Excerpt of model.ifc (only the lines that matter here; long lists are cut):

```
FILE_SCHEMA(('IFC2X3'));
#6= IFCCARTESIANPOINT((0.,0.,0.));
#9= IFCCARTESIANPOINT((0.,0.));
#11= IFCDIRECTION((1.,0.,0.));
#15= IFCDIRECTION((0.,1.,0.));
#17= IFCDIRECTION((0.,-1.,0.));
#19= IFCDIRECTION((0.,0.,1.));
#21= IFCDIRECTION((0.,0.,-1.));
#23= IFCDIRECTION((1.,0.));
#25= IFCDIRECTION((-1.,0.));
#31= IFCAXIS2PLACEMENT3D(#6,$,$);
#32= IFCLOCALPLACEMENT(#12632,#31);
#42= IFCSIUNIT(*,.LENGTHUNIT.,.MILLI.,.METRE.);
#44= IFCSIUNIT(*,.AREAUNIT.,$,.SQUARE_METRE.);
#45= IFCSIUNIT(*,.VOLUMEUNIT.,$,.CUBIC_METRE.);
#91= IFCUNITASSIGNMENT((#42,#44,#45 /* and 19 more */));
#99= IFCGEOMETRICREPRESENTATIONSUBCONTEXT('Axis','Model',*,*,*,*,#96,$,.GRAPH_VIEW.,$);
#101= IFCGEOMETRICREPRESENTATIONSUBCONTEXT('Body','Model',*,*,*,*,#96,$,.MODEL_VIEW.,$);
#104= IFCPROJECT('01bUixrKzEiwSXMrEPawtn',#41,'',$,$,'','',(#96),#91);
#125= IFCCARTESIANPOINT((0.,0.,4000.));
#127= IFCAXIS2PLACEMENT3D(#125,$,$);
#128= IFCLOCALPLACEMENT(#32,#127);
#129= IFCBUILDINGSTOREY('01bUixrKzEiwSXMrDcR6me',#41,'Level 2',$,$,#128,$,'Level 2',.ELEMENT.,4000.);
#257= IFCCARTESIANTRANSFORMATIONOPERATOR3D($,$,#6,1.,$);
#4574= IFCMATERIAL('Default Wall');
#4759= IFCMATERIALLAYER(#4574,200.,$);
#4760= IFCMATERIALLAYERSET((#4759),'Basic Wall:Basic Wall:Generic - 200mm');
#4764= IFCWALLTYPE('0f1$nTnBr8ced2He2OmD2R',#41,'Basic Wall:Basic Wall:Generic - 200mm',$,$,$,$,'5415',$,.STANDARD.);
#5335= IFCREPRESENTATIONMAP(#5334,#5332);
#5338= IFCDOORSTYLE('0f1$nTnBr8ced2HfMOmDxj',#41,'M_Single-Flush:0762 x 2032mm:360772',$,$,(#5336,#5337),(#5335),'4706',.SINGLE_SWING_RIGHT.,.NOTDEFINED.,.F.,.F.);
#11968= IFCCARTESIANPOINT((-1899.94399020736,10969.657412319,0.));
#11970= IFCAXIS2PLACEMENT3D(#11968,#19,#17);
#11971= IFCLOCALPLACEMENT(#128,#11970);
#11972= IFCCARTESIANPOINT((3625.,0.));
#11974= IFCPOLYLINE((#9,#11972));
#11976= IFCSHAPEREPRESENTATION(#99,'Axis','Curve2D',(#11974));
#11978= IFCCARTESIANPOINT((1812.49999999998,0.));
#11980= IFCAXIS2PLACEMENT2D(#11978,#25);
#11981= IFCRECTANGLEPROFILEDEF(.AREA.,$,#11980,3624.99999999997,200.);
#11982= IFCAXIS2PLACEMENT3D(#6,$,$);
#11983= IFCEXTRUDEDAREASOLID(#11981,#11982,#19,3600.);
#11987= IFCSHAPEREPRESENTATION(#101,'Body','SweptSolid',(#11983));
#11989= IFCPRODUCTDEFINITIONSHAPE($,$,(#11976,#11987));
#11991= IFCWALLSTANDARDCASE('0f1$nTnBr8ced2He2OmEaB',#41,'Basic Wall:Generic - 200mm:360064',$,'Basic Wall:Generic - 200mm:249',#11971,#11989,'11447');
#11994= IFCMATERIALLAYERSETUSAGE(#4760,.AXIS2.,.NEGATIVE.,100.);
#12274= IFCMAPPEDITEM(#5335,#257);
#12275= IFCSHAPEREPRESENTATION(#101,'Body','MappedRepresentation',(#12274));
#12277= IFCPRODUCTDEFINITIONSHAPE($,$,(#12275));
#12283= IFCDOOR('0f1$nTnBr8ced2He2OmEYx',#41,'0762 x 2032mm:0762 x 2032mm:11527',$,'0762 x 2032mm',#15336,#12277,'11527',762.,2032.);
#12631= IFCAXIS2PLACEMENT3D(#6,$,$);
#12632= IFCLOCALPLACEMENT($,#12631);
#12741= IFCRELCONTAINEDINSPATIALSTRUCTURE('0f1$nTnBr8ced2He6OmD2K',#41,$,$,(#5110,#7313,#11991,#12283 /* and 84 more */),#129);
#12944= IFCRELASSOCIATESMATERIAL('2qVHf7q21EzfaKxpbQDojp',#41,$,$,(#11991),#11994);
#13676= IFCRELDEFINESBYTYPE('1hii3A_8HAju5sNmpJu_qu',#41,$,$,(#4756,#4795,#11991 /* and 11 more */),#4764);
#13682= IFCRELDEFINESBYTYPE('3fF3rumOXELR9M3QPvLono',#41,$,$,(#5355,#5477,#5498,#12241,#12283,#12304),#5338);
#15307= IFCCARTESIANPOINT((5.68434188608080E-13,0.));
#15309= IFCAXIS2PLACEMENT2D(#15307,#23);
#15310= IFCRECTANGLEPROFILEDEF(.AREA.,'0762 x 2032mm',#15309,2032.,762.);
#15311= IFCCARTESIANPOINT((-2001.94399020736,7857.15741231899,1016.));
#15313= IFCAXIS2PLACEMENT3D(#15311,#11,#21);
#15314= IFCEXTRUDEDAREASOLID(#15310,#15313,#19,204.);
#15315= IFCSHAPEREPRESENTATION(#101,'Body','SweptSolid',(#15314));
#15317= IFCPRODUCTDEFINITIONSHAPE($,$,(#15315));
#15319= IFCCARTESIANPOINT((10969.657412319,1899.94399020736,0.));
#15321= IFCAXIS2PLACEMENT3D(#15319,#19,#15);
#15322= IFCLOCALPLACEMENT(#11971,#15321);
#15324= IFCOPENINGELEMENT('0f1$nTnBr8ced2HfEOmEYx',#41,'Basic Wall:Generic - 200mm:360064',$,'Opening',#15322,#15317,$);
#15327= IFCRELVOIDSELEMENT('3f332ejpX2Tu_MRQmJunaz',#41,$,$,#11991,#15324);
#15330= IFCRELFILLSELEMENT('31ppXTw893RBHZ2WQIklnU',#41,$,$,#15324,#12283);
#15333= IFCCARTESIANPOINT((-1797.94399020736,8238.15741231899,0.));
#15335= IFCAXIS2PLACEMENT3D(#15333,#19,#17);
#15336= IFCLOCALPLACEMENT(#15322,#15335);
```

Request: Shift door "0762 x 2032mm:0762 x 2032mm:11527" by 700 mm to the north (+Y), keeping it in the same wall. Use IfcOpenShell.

```python
import ifcopenshell
import ifcopenshell.api.geometry
import ifcopenshell.util.placement
import ifcopenshell.util.unit

model = ifcopenshell.open("model.ifc")
unit_scale = ifcopenshell.util.unit.calculate_unit_scale(model)

door = model.by_id(12283)
opening = door.FillsVoids[0].RelatingOpeningElement
wall = opening.VoidsElements[0].RelatingBuildingElement

wall_matrix = ifcopenshell.util.placement.get_local_placement(wall.ObjectPlacement)
shift = wall_matrix[:3, 0] * -0.7 / unit_scale
before = ifcopenshell.util.placement.get_local_placement(door.ObjectPlacement)[:3, 3].copy()

# The door is placed relative to its opening, so it follows when the opening moves.
matrix = ifcopenshell.util.placement.get_local_placement(opening.ObjectPlacement)
matrix[:3, 3] += shift
ifcopenshell.api.geometry.edit_object_placement(
    model, product=opening, matrix=matrix, is_si=False, should_transform_children=True
)

after = ifcopenshell.util.placement.get_local_placement(door.ObjectPlacement)[:3, 3]
print("door moved by", (after - before).round(3) + 0.0)

model.write("model_updated.ifc")
```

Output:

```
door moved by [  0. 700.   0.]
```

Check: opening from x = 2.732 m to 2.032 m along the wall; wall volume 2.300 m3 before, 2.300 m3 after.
